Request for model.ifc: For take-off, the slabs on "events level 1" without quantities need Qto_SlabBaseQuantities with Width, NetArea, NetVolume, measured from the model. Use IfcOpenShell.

First a look at what the model holds.

```python
import ifcopenshell
import ifcopenshell.util.element
import ifcopenshell.util.unit

model = ifcopenshell.open("model.ifc")
print(model.schema)
for unit_type in ("LENGTHUNIT", "AREAUNIT", "VOLUMEUNIT"):
    print(unit_type, ifcopenshell.util.unit.calculate_unit_scale(model, unit_type))
storey = next(s for s in model.by_type("IfcBuildingStorey") if s.Name == "events level 1")
slabs = [e for e in ifcopenshell.util.element.get_decomposition(storey) if e.is_a("IfcSlab")]
for e in sorted(slabs, key=lambda e: e.id()):
    print(e.id(), e.is_a(), e.Name, list(ifcopenshell.util.element.get_psets(e, qtos_only=True)), sep=" | ")
```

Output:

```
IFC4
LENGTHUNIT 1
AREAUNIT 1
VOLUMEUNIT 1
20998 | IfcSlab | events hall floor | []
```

```python
import ifcopenshell
import ifcopenshell.api.pset
import ifcopenshell.geom
import ifcopenshell.util.element
import ifcopenshell.util.shape
import ifcopenshell.util.unit

model = ifcopenshell.open("model.ifc")
unit_scale = ifcopenshell.util.unit.calculate_unit_scale(model)
area_scale = ifcopenshell.util.unit.calculate_unit_scale(model, "AREAUNIT")
volume_scale = ifcopenshell.util.unit.calculate_unit_scale(model, "VOLUMEUNIT")
settings = ifcopenshell.geom.settings()

storey = next(s for s in model.by_type("IfcBuildingStorey") if s.Name == "events level 1")
slabs = [e for e in ifcopenshell.util.element.get_decomposition(storey) if e.is_a("IfcSlab")]

for e in sorted(slabs, key=lambda e: e.id()):
    if ifcopenshell.util.element.get_psets(e, qtos_only=True, should_inherit=False):
        continue
    # Geometry comes back in metres, in the element's own axes.
    shape = ifcopenshell.geom.create_shape(settings, e)
    values = {
        "Width": ifcopenshell.util.shape.get_z(shape.geometry) / unit_scale,
        "NetArea": ifcopenshell.util.shape.get_footprint_area(shape.geometry) / area_scale,
        "NetVolume": ifcopenshell.util.shape.get_volume(shape.geometry) / volume_scale,
    }
    qto = ifcopenshell.api.pset.add_qto(model, product=e, name="Qto_SlabBaseQuantities")
    ifcopenshell.api.pset.edit_qto(model, qto=qto, properties=values)
    print(e.id(), {k: round(v, 3) for k, v in values.items()})

model.write("model-out.ifc")
```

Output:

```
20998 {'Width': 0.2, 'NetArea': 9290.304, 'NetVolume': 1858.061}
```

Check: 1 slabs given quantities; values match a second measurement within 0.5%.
